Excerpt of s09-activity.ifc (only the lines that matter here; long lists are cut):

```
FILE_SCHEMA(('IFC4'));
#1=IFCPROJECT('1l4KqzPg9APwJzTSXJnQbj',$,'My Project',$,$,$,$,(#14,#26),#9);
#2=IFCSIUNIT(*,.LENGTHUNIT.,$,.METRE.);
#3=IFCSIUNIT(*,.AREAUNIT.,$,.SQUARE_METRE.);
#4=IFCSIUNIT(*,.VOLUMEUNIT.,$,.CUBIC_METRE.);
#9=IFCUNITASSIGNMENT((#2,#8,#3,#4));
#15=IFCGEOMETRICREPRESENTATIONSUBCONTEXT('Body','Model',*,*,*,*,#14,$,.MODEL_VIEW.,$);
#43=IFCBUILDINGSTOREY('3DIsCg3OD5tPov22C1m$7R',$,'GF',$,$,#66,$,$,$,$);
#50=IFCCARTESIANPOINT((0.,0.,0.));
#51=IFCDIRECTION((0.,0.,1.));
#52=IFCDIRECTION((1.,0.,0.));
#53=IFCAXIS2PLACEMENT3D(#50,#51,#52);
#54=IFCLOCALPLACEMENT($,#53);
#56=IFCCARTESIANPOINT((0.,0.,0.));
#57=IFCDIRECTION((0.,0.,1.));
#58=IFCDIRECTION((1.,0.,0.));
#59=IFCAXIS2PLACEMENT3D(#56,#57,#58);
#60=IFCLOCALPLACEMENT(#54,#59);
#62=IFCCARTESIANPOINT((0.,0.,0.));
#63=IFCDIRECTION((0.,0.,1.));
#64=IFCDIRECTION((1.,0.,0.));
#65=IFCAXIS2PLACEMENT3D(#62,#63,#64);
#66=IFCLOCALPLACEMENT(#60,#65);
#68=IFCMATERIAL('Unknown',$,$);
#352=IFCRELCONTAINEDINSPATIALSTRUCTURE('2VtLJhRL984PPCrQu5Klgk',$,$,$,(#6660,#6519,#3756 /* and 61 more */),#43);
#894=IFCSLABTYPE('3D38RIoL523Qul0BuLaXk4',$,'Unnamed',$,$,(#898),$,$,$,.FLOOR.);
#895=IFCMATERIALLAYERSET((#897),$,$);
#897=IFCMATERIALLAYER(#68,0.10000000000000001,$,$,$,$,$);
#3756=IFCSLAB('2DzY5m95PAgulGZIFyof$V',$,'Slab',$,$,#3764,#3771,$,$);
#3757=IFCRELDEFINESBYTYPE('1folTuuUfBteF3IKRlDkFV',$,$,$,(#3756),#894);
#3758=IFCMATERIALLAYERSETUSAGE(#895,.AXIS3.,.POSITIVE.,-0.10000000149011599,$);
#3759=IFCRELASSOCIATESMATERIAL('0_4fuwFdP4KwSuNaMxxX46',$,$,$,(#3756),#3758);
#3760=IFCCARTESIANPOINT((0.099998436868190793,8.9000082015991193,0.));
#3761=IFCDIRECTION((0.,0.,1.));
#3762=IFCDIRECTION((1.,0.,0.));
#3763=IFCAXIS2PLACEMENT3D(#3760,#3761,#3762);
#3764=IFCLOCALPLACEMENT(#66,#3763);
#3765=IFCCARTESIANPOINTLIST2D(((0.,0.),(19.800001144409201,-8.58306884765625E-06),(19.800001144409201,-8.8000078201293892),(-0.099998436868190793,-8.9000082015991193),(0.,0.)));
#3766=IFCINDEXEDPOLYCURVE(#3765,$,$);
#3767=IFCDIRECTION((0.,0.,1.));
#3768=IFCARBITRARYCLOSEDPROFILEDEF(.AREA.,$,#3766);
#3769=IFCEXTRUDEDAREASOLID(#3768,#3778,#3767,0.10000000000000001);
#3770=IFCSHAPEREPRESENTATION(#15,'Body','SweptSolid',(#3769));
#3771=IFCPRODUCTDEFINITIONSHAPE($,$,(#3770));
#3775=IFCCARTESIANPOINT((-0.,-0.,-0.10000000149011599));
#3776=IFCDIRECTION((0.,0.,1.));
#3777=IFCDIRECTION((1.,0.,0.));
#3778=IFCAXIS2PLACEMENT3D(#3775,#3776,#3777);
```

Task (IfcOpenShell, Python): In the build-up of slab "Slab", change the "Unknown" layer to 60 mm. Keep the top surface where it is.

```python
import ifcopenshell
import ifcopenshell.util.element
import ifcopenshell.util.representation
import ifcopenshell.util.unit

model = ifcopenshell.open("s09-activity.ifc")
unit_scale = ifcopenshell.util.unit.calculate_unit_scale(model)

layer_set = model.by_id(895)
layer = next(l for l in layer_set.MaterialLayers if l.Material and l.Material.Name == "Unknown")
change = 0.06 / unit_scale - layer.LayerThickness
layer.LayerThickness += change

# Geometry does not follow the layer set by itself.
slabs = [e for e in ifcopenshell.util.element.get_elements_by_material(model, layer_set) if e.is_a("IfcSlab")]
for slab in sorted(slabs, key=lambda e: e.id()):
    body = ifcopenshell.util.representation.get_representation(slab, "Model", "Body")
    solid = body.Items[0]
    old_depth = solid.Depth
    solid.Depth += change
    # Extruded upwards: lower the start of the extrusion so the top stays.
    x, y, z = solid.Position.Location.Coordinates
    solid.Position.Location = model.createIfcCartesianPoint((x, y, z - change))
    print(slab.id(), f"{old_depth:g} -> {solid.Depth:g}")

# The layers are counted up from the underside, which has moved.
for usage in {ifcopenshell.util.element.get_material(slab) for slab in slabs}:
    usage.OffsetFromReferenceLine -= change

model.write("s09-activity-out.ifc")
```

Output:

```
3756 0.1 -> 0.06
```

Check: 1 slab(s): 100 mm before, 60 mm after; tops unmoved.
